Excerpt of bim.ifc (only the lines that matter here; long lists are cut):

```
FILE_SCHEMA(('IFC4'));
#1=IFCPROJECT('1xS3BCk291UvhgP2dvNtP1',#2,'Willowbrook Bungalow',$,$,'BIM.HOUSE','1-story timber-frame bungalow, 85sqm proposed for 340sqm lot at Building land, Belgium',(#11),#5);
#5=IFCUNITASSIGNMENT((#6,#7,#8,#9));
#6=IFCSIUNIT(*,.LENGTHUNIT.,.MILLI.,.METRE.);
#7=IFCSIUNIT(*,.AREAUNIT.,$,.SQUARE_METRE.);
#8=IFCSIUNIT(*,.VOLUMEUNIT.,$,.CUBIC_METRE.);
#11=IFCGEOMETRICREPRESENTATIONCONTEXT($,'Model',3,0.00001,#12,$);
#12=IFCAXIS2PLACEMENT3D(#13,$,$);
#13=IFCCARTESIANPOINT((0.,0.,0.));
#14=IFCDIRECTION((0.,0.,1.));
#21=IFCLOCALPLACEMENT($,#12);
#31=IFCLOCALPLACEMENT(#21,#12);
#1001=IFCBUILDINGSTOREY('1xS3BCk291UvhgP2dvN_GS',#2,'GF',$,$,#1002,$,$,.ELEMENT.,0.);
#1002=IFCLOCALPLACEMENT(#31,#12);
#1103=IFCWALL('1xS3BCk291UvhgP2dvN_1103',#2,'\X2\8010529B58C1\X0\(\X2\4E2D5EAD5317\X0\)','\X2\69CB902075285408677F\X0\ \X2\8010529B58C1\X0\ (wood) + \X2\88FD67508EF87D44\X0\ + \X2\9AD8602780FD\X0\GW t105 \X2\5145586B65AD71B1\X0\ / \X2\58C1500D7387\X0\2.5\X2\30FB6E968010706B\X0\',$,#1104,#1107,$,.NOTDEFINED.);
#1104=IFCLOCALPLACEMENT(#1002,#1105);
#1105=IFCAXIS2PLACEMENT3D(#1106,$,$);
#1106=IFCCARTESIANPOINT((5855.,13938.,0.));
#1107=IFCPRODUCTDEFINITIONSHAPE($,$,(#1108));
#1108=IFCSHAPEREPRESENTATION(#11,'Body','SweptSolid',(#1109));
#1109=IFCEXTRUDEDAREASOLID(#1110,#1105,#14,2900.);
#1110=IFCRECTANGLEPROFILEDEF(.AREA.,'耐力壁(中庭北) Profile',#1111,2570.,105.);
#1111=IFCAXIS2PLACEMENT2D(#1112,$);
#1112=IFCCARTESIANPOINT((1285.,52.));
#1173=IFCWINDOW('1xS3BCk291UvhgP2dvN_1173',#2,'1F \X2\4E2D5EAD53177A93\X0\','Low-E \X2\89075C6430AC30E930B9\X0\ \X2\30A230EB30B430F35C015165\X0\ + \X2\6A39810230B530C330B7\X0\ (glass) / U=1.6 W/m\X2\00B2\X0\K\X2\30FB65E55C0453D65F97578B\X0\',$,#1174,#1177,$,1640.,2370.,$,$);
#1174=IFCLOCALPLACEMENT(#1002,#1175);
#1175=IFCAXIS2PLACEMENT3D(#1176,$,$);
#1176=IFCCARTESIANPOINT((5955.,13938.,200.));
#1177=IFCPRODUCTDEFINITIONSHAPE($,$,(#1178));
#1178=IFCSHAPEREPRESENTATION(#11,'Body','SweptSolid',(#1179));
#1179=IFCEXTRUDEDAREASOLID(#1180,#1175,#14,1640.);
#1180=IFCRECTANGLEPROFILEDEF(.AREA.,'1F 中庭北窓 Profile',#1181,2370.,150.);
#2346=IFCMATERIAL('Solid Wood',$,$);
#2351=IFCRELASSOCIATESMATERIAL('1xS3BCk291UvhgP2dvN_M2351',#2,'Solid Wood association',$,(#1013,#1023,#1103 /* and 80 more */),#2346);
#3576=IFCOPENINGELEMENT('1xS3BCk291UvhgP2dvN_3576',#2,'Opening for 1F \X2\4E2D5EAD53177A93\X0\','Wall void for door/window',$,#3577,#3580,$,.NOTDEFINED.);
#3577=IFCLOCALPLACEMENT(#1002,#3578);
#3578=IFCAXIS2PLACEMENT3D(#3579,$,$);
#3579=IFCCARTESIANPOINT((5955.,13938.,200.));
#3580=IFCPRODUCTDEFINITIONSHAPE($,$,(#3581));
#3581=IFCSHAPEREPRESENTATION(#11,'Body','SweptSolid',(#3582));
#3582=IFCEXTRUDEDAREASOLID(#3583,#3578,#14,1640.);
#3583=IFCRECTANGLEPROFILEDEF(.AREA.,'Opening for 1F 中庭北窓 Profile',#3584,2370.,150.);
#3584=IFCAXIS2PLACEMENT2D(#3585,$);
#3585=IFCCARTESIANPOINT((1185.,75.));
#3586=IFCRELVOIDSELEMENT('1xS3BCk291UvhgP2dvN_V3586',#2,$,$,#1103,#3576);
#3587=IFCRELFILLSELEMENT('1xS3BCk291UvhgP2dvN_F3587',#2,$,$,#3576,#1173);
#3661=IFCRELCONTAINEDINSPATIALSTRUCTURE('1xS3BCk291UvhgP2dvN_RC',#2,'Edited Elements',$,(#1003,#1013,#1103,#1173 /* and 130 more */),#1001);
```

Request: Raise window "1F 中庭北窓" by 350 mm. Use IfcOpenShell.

```python
import numpy as np
import ifcopenshell
import ifcopenshell.api.geometry
import ifcopenshell.util.placement
import ifcopenshell.util.unit

model = ifcopenshell.open("bim.ifc")
unit_scale = ifcopenshell.util.unit.calculate_unit_scale(model)

window = model.by_guid("1xS3BCk291UvhgP2dvN_1173")
opening = window.FillsVoids[0].RelatingOpeningElement
dz = 0.35 / unit_scale

shift = np.array([0.0, 0.0, dz])
# The window is not placed relative to its opening, so move both.
for product in (opening, window):
    matrix = ifcopenshell.util.placement.get_local_placement(product.ObjectPlacement)
    matrix[:3, 3] += shift
    ifcopenshell.api.geometry.edit_object_placement(model, product=product, matrix=matrix, is_si=False)

print(f"moved by {dz * unit_scale:+.3f} m")

model.write("bim_v2.ifc")
```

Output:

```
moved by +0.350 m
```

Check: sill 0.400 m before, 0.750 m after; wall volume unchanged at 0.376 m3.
